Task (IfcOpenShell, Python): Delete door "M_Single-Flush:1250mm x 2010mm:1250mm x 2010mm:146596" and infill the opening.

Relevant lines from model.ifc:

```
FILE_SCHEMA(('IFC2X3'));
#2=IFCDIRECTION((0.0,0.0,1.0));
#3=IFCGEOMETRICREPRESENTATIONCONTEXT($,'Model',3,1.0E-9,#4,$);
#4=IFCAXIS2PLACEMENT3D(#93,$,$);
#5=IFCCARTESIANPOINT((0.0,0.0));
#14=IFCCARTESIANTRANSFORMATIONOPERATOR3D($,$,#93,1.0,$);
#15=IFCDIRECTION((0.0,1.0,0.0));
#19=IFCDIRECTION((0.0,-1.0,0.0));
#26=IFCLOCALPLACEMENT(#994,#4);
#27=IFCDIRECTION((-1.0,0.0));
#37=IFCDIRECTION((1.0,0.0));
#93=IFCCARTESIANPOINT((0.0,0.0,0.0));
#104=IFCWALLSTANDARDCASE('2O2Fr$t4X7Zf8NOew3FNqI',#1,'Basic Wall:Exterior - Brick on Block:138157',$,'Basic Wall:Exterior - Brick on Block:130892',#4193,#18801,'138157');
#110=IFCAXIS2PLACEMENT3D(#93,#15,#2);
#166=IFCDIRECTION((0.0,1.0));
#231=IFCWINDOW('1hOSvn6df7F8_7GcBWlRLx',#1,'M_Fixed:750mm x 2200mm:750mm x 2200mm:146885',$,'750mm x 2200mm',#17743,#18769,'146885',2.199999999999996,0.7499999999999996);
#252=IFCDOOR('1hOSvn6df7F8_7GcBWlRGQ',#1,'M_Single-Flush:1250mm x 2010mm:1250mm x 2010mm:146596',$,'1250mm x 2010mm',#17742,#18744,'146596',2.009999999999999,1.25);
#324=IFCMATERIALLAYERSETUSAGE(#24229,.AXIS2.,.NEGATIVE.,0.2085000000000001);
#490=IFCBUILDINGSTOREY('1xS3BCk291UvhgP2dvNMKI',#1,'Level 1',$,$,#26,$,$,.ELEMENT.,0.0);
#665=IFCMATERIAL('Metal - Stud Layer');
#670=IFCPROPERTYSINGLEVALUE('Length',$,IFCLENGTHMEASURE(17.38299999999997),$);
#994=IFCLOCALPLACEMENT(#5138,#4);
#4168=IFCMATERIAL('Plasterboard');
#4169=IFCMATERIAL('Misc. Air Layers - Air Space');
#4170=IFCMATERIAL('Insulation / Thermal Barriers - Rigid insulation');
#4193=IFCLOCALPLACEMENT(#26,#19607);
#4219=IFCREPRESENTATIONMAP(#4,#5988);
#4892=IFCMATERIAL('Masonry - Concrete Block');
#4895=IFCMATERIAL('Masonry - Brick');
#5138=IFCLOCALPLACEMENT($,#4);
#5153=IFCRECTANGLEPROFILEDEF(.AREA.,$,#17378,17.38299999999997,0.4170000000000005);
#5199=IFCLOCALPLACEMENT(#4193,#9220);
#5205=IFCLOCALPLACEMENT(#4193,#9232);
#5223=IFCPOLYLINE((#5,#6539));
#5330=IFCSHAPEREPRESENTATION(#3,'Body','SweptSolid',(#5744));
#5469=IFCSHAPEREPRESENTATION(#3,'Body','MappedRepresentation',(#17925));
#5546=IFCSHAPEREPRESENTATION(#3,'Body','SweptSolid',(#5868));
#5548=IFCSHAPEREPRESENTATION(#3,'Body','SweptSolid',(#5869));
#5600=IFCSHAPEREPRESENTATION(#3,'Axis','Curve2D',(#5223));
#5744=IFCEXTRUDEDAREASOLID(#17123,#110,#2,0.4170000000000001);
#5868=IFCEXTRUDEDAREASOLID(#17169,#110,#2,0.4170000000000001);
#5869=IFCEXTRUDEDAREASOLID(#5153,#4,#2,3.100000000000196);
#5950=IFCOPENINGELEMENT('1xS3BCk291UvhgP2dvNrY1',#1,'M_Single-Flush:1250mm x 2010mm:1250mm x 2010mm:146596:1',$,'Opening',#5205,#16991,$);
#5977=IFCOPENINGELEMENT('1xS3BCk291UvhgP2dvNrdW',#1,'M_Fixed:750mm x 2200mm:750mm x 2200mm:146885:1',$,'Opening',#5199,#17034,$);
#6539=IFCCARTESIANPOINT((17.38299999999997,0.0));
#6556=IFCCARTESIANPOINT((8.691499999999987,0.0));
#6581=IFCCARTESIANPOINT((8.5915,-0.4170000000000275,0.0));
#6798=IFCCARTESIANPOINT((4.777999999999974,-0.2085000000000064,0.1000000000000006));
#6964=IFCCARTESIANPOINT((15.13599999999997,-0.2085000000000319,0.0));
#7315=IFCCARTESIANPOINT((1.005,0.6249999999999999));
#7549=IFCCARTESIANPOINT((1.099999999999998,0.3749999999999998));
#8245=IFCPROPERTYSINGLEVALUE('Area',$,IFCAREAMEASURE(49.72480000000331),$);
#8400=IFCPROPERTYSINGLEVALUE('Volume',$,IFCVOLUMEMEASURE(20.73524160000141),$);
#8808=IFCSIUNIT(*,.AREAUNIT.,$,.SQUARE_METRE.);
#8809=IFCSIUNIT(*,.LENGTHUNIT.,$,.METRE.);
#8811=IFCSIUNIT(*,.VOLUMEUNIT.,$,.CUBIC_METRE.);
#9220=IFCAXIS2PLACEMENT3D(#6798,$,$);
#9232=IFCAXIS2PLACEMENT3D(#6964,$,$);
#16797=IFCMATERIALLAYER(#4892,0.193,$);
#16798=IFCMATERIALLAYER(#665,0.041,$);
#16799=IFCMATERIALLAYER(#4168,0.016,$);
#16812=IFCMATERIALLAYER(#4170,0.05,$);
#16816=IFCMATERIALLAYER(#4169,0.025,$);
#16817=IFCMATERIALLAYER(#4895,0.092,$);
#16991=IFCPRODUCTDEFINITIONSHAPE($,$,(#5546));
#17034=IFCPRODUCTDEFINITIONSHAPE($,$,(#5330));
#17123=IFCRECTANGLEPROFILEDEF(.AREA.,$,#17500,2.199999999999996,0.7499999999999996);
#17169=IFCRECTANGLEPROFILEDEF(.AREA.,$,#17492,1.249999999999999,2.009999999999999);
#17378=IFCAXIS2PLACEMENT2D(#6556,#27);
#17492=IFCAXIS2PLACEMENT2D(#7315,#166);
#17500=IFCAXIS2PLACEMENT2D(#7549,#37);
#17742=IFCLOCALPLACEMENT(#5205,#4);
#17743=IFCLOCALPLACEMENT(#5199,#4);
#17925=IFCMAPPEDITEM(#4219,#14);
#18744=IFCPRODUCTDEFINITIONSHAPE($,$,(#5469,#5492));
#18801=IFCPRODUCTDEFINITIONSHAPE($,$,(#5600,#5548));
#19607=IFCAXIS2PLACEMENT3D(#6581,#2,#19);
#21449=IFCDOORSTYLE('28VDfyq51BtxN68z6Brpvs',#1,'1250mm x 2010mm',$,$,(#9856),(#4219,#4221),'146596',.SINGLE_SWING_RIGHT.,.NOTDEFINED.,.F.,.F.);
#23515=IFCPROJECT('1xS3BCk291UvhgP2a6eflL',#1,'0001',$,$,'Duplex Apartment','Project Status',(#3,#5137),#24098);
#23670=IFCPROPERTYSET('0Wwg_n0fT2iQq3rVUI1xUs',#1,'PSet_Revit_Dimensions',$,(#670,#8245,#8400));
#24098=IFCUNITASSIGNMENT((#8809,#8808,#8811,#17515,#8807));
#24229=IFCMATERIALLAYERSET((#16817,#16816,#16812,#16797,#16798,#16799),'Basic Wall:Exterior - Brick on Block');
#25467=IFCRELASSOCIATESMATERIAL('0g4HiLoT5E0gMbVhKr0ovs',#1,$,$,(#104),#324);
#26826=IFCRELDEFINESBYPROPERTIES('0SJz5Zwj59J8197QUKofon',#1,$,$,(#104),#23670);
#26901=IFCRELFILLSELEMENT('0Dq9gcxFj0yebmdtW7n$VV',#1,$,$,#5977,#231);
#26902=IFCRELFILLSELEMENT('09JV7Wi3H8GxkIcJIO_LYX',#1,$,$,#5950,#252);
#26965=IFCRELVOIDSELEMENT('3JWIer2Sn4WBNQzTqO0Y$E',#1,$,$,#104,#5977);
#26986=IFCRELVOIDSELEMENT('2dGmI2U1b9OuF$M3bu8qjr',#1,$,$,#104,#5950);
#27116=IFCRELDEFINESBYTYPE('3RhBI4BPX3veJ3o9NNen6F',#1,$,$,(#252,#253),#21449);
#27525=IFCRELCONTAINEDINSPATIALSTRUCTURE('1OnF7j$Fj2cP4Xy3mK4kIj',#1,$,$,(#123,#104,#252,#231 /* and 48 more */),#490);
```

```python
import ifcopenshell
import ifcopenshell.api.feature
import ifcopenshell.api.pset
import ifcopenshell.api.root
import ifcopenshell.geom
import ifcopenshell.util.element
import ifcopenshell.util.shape
import ifcopenshell.util.unit

model = ifcopenshell.open("model.ifc")
area_scale = ifcopenshell.util.unit.calculate_unit_scale(model, "AREAUNIT")
volume_scale = ifcopenshell.util.unit.calculate_unit_scale(model, "VOLUMEUNIT")
settings = ifcopenshell.geom.settings()


def volume(element):
    """Net volume in cubic metres, openings subtracted."""
    shape = ifcopenshell.geom.create_shape(settings, element)
    return ifcopenshell.util.shape.get_volume(shape.geometry)


door = model.by_guid("1hOSvn6df7F8_7GcBWlRGQ")
opening = door.FillsVoids[0].RelatingOpeningElement
wall = opening.VoidsElements[0].RelatingBuildingElement
before = volume(wall)

ifcopenshell.api.root.remove_product(model, product=door)
ifcopenshell.api.feature.remove_feature(model, feature=opening)

after = volume(wall)
thickness = 0.417  # wall thickness in metres

# Update the wall's stored quantities.
pset = model.by_id(ifcopenshell.util.element.get_pset(wall, "PSet_Revit_Dimensions", should_inherit=False)["id"])
ifcopenshell.api.pset.edit_pset(model, pset=pset, properties={
    "Area": model.create_entity("IfcAreaMeasure", after / thickness / area_scale),
    "Volume": model.create_entity("IfcVolumeMeasure", after / volume_scale),
})

print(f"wall volume {before:.3f} -> {after:.3f} m3")

model.write("model_rev.ifc")
```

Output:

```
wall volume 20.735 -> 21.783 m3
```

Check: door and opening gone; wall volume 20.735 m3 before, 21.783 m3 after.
